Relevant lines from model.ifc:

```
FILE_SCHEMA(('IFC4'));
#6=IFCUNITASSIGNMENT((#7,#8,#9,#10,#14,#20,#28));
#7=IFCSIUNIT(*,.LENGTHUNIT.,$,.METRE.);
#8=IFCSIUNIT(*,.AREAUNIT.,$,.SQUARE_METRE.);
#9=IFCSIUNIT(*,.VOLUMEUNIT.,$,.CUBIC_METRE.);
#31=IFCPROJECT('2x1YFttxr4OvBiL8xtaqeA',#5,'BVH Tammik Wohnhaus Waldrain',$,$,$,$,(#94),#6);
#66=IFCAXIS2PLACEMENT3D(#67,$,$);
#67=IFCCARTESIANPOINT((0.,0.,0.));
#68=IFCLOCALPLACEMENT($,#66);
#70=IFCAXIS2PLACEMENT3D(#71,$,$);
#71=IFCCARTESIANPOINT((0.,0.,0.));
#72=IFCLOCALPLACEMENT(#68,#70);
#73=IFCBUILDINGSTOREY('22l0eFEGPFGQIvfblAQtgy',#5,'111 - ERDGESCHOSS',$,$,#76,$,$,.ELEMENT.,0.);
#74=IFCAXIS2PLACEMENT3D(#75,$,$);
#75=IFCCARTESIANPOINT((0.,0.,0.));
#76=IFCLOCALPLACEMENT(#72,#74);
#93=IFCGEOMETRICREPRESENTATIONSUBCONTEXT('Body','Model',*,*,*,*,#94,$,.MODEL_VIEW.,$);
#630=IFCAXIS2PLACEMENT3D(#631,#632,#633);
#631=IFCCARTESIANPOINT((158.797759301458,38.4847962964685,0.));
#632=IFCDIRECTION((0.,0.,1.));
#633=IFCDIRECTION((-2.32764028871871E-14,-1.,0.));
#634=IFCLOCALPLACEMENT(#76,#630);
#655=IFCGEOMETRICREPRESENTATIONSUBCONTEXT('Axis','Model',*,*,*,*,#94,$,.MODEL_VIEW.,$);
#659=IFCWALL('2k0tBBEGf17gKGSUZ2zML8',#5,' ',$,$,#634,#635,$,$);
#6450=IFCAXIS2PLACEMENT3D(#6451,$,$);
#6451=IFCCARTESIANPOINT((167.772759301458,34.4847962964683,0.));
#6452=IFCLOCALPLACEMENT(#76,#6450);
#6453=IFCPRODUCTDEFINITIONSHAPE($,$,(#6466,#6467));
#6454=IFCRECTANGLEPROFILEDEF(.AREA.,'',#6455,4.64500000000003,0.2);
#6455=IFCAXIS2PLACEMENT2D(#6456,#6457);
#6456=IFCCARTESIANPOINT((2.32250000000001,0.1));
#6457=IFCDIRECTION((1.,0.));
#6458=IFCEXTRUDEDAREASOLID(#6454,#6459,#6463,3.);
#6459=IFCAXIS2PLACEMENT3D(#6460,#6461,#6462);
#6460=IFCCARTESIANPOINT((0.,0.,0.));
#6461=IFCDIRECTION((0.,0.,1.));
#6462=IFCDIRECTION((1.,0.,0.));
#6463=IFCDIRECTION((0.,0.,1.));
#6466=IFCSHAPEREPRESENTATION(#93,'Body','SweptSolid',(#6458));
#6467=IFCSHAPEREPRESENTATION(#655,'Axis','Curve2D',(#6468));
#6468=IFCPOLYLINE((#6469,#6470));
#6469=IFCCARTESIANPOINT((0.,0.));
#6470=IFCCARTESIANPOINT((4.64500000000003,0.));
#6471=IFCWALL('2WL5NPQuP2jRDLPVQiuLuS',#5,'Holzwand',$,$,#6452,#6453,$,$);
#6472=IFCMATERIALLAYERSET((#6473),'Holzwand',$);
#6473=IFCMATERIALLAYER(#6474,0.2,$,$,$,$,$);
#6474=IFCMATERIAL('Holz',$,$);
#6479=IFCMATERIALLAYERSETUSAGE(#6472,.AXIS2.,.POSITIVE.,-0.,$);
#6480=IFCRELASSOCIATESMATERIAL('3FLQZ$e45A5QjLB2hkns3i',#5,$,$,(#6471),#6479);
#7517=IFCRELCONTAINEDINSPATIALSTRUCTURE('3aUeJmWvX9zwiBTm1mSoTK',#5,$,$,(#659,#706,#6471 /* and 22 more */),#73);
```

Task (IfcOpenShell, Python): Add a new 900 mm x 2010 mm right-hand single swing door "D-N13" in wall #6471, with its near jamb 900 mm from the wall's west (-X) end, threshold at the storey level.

```python
import numpy as np
import ifcopenshell
import ifcopenshell.api.feature
import ifcopenshell.api.geometry
import ifcopenshell.api.root
import ifcopenshell.api.spatial
import ifcopenshell.geom
import ifcopenshell.util.element
import ifcopenshell.util.placement
import ifcopenshell.util.representation
import ifcopenshell.util.shape
import ifcopenshell.util.unit

model = ifcopenshell.open("model.ifc")
unit_scale = ifcopenshell.util.unit.calculate_unit_scale(model)
settings = ifcopenshell.geom.settings()


def volume(element):
    """Net volume in cubic metres, openings subtracted."""
    shape = ifcopenshell.geom.create_shape(settings, element)
    return ifcopenshell.util.shape.get_volume(shape.geometry)


wall = model.by_id(6471)
storey = ifcopenshell.util.element.get_container(wall, ifc_class="IfcBuildingStorey")
context = ifcopenshell.util.representation.get_context(model, "Model", "Body", "MODEL_VIEW")
before = volume(wall)

width, height, from_end, sill = 0.9, 2.01, 0.9, 0.0  # metres

# The wall runs along its own X axis, and the end named is its -X end.
wall_shape = ifcopenshell.geom.create_shape(settings, wall)
x, y, z = ifcopenshell.util.shape.get_vertices(wall_shape.geometry).T
start = x.min() + from_end
face, thickness = float(y.min()), float(y.max() - y.min())
wall_matrix = ifcopenshell.util.placement.get_local_placement(wall.ObjectPlacement)
level = ifcopenshell.util.placement.get_local_placement(storey.ObjectPlacement)[2, 3]


def in_wall(x, y):
    """Placement at x, y metres in the wall's axes, at sill height."""
    matrix = wall_matrix.copy()
    matrix[:, 3] = wall_matrix @ np.array([x / unit_scale, y / unit_scale, 0.0, 1.0])
    matrix[2, 3] = level + sill / unit_scale
    return matrix


# Opening: a box that overshoots both wall faces by 50 mm.
opening = ifcopenshell.api.root.create_entity(model, ifc_class="IfcOpeningElement", predefined_type="OPENING")
box = ifcopenshell.api.geometry.add_wall_representation(
    model, context=context, length=width, height=height, thickness=thickness + 0.1
)
ifcopenshell.api.geometry.assign_representation(model, product=opening, representation=box)
ifcopenshell.api.geometry.edit_object_placement(model, product=opening, matrix=in_wall(start, face - 0.05), is_si=False)
ifcopenshell.api.feature.add_feature(model, feature=opening, element=wall)

door = ifcopenshell.api.root.create_entity(model, ifc_class="IfcDoor", name="D-N13", predefined_type="DOOR")
door.OverallWidth, door.OverallHeight = width / unit_scale, height / unit_scale
door.OperationType = "SINGLE_SWING_RIGHT"
body = ifcopenshell.api.geometry.add_door_representation(
    model,
    context=context,
    overall_width=door.OverallWidth,
    overall_height=door.OverallHeight,
    operation_type="SINGLE_SWING_RIGHT",
    lining_properties={"LiningDepth": thickness / unit_scale, "ThresholdDepth": thickness / unit_scale},
)
ifcopenshell.api.geometry.assign_representation(model, product=door, representation=body)
ifcopenshell.api.spatial.assign_container(model, products=[door], relating_structure=storey)
ifcopenshell.api.feature.add_filling(model, opening=opening, element=door)

# The lining spans the wall, so the door starts at the wall face.
ifcopenshell.api.geometry.edit_object_placement(model, product=door, matrix=in_wall(start, face), is_si=False)

after = volume(wall)

print(f"wall volume {before:.3f} -> {after:.3f} m3")

model.write("model_rev.ifc")
```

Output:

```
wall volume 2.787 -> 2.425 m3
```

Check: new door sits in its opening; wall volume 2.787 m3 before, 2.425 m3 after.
